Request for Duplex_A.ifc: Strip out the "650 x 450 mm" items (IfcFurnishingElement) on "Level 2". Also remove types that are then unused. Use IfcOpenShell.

First a look at what the model holds.

```python
import ifcopenshell
import ifcopenshell.util.element

model = ifcopenshell.open("Duplex_A.ifc")
print(model.schema)
storey = next(s for s in model.by_type("IfcBuildingStorey") if s.Name == "Level 2")
furniture = [e for e in ifcopenshell.util.element.get_decomposition(storey) if e.is_a("IfcFurnishingElement")]
seen = {}
for e in furniture:
    element_type = ifcopenshell.util.element.get_type(e)
    name = element_type.Name if element_type not in (None, e) else None
    seen[name] = seen.get(name, 0) + 1
for name, count in sorted(seen.items(), key=str):
    print(count, "x", name)
```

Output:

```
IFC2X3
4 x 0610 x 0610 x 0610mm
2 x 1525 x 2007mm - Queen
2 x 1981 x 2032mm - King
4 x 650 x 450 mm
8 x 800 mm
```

```python
import ifcopenshell
import ifcopenshell.api.root
import ifcopenshell.util.element

model = ifcopenshell.open("Duplex_A.ifc")

storey = next(s for s in model.by_type("IfcBuildingStorey") if s.Name == "Level 2")
furniture = [e for e in ifcopenshell.util.element.get_decomposition(storey) if e.is_a("IfcFurnishingElement")]
targets = [e for e in furniture if (t := ifcopenshell.util.element.get_type(e)) not in (None, e) and t.Name == "650 x 450 mm"]
types = {ifcopenshell.util.element.get_type(e) for e in targets} - {None, *targets}

for e in targets:
    ifcopenshell.api.root.remove_product(model, product=e)
print(len(targets), "removed")

unused = [t for t in types if not ifcopenshell.util.element.get_types(t)]
for t in unused:
    ifcopenshell.api.root.remove_product(model, product=t)
print(len(unused), "unused types removed")

model.write("Duplex_A_edited.ifc")
```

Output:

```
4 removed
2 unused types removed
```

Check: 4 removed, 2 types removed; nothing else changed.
